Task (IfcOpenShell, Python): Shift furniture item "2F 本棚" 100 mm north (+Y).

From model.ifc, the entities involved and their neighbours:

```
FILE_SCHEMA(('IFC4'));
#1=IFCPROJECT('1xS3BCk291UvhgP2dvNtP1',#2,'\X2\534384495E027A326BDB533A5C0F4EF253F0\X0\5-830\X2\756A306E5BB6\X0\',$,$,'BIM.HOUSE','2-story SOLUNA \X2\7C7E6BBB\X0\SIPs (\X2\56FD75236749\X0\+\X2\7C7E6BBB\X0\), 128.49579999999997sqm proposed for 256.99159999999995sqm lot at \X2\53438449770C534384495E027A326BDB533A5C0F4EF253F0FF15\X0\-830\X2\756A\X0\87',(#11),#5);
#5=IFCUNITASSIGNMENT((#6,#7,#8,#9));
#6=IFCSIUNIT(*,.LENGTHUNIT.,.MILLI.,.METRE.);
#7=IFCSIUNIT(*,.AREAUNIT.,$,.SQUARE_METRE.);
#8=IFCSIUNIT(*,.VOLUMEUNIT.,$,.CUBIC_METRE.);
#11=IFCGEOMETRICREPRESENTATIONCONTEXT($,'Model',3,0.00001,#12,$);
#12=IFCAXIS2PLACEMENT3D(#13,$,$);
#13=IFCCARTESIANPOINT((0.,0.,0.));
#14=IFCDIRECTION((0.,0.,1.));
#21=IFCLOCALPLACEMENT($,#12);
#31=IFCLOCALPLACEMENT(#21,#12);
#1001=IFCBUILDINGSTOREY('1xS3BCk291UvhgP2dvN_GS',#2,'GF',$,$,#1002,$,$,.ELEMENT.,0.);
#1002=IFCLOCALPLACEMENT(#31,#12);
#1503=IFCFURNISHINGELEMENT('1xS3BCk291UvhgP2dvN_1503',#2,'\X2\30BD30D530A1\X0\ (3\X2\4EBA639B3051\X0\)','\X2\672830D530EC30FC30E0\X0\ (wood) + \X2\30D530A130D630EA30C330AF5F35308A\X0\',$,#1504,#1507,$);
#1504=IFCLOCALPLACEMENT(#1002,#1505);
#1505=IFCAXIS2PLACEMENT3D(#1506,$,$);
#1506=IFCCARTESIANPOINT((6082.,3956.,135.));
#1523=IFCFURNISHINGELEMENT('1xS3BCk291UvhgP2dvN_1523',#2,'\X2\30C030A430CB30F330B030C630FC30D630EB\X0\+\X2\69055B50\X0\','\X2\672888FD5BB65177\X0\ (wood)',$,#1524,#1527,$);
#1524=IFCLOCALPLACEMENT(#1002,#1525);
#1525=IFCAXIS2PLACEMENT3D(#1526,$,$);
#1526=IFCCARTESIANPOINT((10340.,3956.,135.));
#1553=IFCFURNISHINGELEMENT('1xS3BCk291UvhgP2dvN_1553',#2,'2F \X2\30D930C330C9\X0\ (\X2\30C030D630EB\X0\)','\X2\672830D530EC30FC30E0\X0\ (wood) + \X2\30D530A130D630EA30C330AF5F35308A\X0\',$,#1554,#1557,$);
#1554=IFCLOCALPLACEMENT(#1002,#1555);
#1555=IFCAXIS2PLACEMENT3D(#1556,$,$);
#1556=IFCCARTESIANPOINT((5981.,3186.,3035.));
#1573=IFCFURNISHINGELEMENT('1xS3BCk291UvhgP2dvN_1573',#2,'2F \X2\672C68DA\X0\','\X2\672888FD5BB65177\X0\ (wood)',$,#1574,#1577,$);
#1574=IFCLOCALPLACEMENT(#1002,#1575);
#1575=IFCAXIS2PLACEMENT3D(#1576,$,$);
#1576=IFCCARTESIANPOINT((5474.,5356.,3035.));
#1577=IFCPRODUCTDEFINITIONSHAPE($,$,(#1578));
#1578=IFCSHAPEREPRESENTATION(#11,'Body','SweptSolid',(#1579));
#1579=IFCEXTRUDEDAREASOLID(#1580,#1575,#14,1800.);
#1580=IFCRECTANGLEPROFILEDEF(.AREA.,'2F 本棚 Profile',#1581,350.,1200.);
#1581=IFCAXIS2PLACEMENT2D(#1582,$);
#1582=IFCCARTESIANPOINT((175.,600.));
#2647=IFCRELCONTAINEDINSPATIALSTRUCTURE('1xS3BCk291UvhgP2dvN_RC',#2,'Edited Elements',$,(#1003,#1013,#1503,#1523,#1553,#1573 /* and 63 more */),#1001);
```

```python
import ifcopenshell
import ifcopenshell.api.geometry
import ifcopenshell.util.placement

model = ifcopenshell.open("model.ifc")

item = model.by_id(1573)
matrix = ifcopenshell.util.placement.get_local_placement(item.ObjectPlacement)
matrix[1, 3] += 100.0
ifcopenshell.api.geometry.edit_object_placement(model, product=item, matrix=matrix, is_si=False)

print(ifcopenshell.util.placement.get_local_placement(item.ObjectPlacement).round(3) + 0.0)

model.write("model_updated.ifc")
```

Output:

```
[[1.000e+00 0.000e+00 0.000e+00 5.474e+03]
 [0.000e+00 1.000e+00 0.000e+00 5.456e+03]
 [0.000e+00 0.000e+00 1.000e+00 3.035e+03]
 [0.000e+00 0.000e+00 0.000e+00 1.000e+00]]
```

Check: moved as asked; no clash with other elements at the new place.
